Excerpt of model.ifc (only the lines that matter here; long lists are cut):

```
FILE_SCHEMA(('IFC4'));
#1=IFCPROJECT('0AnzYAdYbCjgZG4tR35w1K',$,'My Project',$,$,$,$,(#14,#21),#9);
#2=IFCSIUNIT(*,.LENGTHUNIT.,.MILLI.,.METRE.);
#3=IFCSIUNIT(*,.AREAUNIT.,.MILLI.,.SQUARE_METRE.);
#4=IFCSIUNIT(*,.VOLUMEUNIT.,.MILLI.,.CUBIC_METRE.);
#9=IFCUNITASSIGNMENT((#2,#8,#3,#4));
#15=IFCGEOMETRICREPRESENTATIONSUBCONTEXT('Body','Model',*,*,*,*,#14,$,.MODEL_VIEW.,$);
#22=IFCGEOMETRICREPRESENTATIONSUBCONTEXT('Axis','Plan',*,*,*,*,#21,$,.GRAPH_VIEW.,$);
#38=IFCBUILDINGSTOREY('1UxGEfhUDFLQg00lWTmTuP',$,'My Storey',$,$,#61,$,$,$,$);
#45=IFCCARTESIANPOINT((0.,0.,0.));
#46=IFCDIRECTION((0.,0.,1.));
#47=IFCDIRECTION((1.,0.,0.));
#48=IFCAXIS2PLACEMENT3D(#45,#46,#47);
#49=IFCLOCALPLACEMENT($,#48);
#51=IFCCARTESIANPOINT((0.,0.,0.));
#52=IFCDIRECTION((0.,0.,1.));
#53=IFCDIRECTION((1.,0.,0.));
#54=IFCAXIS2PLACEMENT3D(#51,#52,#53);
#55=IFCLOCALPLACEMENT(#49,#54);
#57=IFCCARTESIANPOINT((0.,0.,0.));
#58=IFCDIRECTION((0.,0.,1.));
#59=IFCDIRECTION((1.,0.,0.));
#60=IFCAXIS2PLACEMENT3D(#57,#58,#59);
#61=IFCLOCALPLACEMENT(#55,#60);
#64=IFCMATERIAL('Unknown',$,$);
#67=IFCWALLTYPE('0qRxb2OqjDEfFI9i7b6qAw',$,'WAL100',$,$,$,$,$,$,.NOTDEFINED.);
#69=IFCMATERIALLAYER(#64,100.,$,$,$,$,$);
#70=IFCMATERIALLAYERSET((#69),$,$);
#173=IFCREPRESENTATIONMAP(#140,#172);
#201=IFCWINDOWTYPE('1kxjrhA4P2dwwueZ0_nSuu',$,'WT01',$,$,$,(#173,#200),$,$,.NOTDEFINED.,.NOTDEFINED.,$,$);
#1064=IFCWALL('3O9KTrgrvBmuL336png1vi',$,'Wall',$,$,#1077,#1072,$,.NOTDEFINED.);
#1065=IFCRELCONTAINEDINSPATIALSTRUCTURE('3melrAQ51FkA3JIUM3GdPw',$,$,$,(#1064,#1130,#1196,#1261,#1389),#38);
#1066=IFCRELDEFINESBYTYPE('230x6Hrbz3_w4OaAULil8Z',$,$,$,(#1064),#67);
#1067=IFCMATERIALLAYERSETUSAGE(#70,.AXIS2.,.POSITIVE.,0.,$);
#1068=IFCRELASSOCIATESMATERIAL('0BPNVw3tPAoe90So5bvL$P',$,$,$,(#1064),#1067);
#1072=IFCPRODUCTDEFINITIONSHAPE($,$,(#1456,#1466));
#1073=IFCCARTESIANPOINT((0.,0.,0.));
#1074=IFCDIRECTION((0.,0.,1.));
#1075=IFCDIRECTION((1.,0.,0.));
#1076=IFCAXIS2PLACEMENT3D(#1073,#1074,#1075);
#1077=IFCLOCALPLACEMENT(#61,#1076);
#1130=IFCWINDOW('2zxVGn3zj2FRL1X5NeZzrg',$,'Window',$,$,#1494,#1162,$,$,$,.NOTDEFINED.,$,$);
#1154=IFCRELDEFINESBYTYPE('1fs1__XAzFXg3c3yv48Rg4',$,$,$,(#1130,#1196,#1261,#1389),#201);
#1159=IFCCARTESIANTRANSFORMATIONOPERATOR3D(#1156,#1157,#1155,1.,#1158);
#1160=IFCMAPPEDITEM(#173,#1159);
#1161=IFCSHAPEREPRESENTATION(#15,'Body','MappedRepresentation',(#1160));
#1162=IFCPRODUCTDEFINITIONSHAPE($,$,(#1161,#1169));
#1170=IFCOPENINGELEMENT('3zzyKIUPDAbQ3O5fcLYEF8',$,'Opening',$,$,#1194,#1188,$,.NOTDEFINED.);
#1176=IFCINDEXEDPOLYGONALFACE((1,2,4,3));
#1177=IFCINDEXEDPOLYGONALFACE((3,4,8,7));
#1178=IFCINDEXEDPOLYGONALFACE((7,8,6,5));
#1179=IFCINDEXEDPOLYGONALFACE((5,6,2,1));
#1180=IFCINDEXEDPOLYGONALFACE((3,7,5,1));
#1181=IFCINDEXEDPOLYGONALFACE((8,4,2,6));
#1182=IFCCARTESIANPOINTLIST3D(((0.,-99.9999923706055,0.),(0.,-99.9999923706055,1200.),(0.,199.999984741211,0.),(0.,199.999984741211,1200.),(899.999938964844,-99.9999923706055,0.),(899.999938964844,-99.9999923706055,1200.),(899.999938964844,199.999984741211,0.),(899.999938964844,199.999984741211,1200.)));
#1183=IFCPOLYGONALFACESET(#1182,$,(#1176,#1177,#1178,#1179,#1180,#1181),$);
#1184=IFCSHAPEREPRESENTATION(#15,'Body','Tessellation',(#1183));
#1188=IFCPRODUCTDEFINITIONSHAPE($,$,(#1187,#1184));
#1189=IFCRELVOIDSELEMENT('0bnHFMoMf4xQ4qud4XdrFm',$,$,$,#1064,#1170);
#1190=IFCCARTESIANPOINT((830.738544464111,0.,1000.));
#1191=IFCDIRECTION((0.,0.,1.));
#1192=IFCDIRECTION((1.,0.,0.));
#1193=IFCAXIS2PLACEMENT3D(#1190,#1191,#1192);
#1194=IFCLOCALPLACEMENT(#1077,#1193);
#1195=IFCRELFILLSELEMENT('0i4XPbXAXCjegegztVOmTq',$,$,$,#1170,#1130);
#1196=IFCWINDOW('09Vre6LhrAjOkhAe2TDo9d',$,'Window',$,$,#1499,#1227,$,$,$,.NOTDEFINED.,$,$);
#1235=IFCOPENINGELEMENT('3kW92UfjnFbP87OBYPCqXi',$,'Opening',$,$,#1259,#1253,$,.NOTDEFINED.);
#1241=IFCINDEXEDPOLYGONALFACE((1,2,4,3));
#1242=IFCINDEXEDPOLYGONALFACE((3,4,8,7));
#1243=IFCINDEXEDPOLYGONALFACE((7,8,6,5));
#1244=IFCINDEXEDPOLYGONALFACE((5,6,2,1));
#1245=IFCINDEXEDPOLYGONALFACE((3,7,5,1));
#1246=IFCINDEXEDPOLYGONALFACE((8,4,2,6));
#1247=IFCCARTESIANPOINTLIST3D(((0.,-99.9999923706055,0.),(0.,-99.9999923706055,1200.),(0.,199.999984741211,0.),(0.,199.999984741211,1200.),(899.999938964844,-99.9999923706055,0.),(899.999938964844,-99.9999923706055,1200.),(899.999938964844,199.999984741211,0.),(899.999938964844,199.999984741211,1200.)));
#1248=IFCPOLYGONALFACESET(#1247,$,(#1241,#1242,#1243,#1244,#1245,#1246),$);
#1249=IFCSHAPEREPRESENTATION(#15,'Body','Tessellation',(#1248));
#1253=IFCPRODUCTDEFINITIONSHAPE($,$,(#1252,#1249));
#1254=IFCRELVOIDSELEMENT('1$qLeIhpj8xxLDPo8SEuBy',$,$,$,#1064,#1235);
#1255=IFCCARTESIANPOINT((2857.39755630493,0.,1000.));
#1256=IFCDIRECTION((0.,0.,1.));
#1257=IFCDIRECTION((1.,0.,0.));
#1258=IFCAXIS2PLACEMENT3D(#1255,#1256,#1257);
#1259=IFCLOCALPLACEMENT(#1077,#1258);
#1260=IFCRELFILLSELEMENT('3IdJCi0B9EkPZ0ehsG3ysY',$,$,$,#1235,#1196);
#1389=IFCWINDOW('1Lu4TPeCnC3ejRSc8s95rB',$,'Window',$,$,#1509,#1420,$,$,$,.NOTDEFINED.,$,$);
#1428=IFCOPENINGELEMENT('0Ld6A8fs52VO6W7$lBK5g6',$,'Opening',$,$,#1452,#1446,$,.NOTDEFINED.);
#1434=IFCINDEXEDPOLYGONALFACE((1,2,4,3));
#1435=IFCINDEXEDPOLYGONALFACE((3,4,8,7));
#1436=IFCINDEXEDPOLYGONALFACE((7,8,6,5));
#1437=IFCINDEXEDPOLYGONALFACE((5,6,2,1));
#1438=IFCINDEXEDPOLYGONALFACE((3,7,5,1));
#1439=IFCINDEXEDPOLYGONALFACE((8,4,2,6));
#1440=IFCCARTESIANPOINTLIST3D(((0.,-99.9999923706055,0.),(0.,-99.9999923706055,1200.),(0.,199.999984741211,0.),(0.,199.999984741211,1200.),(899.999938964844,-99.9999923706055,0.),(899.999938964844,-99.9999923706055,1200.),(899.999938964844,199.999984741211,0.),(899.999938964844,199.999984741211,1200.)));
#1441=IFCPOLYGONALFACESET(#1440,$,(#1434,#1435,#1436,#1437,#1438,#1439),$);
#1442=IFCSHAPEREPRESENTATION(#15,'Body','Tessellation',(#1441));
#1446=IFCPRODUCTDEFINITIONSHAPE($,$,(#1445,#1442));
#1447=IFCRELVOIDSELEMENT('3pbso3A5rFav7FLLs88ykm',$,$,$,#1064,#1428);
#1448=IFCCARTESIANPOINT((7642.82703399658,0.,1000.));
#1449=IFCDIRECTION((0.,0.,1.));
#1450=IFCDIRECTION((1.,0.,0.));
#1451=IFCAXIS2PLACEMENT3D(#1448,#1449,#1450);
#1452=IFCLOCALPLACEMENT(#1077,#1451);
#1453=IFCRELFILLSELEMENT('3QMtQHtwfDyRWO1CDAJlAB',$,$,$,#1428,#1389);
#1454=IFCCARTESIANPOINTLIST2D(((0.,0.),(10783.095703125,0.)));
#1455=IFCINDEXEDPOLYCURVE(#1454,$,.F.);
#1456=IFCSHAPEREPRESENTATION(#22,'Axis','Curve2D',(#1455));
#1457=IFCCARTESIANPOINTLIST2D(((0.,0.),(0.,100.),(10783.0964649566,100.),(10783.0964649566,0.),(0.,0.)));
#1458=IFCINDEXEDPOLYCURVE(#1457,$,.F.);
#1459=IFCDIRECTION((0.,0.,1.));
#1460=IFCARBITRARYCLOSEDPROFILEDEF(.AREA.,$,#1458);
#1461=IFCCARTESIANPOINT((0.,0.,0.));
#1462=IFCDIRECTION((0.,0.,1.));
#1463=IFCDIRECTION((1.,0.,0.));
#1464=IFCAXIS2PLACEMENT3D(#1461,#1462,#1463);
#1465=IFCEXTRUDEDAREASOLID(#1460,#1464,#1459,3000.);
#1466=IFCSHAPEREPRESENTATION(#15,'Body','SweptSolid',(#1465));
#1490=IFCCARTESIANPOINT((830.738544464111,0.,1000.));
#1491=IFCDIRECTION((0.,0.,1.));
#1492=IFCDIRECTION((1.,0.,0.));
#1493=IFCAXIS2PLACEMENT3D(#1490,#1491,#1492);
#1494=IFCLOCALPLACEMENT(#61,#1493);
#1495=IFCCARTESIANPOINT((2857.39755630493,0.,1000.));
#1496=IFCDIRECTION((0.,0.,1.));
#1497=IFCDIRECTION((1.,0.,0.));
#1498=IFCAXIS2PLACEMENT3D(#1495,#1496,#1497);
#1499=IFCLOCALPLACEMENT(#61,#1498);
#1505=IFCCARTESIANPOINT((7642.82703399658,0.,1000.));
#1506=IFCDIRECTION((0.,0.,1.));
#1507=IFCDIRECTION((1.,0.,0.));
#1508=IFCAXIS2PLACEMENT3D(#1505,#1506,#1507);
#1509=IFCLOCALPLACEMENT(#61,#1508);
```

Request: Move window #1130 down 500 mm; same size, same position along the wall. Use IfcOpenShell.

```python
import numpy as np
import ifcopenshell
import ifcopenshell.api.geometry
import ifcopenshell.util.placement
import ifcopenshell.util.unit

model = ifcopenshell.open("model.ifc")
unit_scale = ifcopenshell.util.unit.calculate_unit_scale(model)

window = model.by_guid("2zxVGn3zj2FRL1X5NeZzrg")
opening = window.FillsVoids[0].RelatingOpeningElement
dz = -0.5 / unit_scale

shift = np.array([0.0, 0.0, dz])
# The window is not placed relative to its opening, so move both.
for product in (opening, window):
    matrix = ifcopenshell.util.placement.get_local_placement(product.ObjectPlacement)
    matrix[:3, 3] += shift
    ifcopenshell.api.geometry.edit_object_placement(model, product=product, matrix=matrix, is_si=False)

print(f"moved by {dz * unit_scale:+.3f} m")

model.write("model_edited.ifc")
```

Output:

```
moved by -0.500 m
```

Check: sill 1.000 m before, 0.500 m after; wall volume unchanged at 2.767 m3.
